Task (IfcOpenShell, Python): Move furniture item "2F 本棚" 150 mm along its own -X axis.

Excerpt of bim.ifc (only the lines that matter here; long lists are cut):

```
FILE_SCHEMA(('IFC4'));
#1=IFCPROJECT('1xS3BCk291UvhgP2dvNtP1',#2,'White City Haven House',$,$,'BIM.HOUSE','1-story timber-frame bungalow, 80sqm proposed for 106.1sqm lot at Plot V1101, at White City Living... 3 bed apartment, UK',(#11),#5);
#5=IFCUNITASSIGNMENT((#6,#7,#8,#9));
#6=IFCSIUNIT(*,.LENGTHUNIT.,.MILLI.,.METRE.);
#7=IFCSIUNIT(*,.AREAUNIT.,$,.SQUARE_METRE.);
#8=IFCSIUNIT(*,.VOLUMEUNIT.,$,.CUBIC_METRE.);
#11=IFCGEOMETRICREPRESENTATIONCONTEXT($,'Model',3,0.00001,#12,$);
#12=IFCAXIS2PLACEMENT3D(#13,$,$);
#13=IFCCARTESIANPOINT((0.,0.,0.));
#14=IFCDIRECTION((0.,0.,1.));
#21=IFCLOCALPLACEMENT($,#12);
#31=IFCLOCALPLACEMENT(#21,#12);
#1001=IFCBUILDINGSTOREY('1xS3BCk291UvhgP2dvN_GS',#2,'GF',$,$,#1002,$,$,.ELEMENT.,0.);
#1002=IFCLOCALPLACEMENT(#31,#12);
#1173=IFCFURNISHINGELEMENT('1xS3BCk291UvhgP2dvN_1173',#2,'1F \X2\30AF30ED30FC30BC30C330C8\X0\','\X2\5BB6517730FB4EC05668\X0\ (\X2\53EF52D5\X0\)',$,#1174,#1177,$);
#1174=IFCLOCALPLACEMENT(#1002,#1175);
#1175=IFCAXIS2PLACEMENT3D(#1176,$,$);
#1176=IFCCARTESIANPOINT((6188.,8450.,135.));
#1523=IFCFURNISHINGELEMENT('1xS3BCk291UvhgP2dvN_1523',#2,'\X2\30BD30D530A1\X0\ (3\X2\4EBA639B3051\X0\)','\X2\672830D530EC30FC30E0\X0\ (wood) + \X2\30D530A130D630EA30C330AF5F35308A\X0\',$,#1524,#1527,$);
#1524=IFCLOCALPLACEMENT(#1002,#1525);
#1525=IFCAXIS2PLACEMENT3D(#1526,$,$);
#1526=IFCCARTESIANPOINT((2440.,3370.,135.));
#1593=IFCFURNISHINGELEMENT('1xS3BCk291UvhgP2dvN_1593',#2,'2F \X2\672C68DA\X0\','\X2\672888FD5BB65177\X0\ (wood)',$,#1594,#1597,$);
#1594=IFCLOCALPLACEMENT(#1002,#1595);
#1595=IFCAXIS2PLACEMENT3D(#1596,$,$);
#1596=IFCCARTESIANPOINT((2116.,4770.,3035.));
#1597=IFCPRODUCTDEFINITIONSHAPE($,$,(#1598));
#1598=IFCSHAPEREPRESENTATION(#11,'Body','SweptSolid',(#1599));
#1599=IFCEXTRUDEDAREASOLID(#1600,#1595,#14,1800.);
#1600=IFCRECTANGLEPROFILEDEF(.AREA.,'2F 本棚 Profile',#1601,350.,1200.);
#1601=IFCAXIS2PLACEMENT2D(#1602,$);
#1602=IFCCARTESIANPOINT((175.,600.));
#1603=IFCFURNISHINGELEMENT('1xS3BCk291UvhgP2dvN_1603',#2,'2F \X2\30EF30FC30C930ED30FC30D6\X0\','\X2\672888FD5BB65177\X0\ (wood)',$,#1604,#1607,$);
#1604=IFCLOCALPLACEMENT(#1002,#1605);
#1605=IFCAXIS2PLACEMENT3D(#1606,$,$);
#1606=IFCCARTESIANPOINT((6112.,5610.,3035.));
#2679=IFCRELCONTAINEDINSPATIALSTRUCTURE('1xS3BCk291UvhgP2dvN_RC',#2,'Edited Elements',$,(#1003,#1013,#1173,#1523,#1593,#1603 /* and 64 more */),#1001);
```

```python
import ifcopenshell
import ifcopenshell.api.geometry
import ifcopenshell.util.placement
import ifcopenshell.util.unit

model = ifcopenshell.open("bim.ifc")
unit_scale = ifcopenshell.util.unit.calculate_unit_scale(model)

item = model.by_id(1593)
matrix = ifcopenshell.util.placement.get_local_placement(item.ObjectPlacement)
matrix[:3, 3] -= matrix[:3, 0] * 0.15 / unit_scale
ifcopenshell.api.geometry.edit_object_placement(model, product=item, matrix=matrix, is_si=False)

print(ifcopenshell.util.placement.get_local_placement(item.ObjectPlacement).round(3) + 0.0)

model.write("bim_v2.ifc")
```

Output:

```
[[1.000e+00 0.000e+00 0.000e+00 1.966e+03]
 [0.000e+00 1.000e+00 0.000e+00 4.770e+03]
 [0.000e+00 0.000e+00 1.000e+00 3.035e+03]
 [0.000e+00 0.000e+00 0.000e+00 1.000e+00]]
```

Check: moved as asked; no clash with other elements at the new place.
